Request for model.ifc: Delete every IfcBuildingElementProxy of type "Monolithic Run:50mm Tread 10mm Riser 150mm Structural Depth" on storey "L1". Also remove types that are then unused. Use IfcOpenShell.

First a look at what the model holds.

```python
import ifcopenshell
import ifcopenshell.util.element

model = ifcopenshell.open("model.ifc")
print(model.schema)
storey = next(s for s in model.by_type("IfcBuildingStorey") if s.Name == "L1")
proxies = [e for e in ifcopenshell.util.element.get_decomposition(storey) if e.is_a("IfcBuildingElementProxy")]
seen = {}
for e in proxies:
    element_type = ifcopenshell.util.element.get_type(e)
    name = element_type.Name if element_type not in (None, e) else None
    seen[name] = seen.get(name, 0) + 1
for name, count in sorted(seen.items(), key=str):
    print(count, "x", name)
```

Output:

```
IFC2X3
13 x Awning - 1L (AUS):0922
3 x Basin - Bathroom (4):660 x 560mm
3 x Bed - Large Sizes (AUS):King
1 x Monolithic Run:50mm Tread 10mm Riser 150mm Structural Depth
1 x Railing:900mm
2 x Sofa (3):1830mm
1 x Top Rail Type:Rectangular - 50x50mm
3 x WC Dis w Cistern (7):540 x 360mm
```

```python
import ifcopenshell
import ifcopenshell.api.root
import ifcopenshell.util.element

model = ifcopenshell.open("model.ifc")

storey = next(s for s in model.by_type("IfcBuildingStorey") if s.Name == "L1")
proxies = [e for e in ifcopenshell.util.element.get_decomposition(storey) if e.is_a("IfcBuildingElementProxy")]
targets = [e for e in proxies if (t := ifcopenshell.util.element.get_type(e)) not in (None, e) and t.Name == "Monolithic Run:50mm Tread 10mm Riser 150mm Structural Depth"]
types = {ifcopenshell.util.element.get_type(e) for e in targets} - {None, *targets}

for e in targets:
    ifcopenshell.api.root.remove_product(model, product=e)
print(len(targets), "removed")

unused = [t for t in types if not ifcopenshell.util.element.get_types(t)]
for t in unused:
    ifcopenshell.api.root.remove_product(model, product=t)
print(len(unused), "unused types removed")

model.write("model_edited.ifc")
```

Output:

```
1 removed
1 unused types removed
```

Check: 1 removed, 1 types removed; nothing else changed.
